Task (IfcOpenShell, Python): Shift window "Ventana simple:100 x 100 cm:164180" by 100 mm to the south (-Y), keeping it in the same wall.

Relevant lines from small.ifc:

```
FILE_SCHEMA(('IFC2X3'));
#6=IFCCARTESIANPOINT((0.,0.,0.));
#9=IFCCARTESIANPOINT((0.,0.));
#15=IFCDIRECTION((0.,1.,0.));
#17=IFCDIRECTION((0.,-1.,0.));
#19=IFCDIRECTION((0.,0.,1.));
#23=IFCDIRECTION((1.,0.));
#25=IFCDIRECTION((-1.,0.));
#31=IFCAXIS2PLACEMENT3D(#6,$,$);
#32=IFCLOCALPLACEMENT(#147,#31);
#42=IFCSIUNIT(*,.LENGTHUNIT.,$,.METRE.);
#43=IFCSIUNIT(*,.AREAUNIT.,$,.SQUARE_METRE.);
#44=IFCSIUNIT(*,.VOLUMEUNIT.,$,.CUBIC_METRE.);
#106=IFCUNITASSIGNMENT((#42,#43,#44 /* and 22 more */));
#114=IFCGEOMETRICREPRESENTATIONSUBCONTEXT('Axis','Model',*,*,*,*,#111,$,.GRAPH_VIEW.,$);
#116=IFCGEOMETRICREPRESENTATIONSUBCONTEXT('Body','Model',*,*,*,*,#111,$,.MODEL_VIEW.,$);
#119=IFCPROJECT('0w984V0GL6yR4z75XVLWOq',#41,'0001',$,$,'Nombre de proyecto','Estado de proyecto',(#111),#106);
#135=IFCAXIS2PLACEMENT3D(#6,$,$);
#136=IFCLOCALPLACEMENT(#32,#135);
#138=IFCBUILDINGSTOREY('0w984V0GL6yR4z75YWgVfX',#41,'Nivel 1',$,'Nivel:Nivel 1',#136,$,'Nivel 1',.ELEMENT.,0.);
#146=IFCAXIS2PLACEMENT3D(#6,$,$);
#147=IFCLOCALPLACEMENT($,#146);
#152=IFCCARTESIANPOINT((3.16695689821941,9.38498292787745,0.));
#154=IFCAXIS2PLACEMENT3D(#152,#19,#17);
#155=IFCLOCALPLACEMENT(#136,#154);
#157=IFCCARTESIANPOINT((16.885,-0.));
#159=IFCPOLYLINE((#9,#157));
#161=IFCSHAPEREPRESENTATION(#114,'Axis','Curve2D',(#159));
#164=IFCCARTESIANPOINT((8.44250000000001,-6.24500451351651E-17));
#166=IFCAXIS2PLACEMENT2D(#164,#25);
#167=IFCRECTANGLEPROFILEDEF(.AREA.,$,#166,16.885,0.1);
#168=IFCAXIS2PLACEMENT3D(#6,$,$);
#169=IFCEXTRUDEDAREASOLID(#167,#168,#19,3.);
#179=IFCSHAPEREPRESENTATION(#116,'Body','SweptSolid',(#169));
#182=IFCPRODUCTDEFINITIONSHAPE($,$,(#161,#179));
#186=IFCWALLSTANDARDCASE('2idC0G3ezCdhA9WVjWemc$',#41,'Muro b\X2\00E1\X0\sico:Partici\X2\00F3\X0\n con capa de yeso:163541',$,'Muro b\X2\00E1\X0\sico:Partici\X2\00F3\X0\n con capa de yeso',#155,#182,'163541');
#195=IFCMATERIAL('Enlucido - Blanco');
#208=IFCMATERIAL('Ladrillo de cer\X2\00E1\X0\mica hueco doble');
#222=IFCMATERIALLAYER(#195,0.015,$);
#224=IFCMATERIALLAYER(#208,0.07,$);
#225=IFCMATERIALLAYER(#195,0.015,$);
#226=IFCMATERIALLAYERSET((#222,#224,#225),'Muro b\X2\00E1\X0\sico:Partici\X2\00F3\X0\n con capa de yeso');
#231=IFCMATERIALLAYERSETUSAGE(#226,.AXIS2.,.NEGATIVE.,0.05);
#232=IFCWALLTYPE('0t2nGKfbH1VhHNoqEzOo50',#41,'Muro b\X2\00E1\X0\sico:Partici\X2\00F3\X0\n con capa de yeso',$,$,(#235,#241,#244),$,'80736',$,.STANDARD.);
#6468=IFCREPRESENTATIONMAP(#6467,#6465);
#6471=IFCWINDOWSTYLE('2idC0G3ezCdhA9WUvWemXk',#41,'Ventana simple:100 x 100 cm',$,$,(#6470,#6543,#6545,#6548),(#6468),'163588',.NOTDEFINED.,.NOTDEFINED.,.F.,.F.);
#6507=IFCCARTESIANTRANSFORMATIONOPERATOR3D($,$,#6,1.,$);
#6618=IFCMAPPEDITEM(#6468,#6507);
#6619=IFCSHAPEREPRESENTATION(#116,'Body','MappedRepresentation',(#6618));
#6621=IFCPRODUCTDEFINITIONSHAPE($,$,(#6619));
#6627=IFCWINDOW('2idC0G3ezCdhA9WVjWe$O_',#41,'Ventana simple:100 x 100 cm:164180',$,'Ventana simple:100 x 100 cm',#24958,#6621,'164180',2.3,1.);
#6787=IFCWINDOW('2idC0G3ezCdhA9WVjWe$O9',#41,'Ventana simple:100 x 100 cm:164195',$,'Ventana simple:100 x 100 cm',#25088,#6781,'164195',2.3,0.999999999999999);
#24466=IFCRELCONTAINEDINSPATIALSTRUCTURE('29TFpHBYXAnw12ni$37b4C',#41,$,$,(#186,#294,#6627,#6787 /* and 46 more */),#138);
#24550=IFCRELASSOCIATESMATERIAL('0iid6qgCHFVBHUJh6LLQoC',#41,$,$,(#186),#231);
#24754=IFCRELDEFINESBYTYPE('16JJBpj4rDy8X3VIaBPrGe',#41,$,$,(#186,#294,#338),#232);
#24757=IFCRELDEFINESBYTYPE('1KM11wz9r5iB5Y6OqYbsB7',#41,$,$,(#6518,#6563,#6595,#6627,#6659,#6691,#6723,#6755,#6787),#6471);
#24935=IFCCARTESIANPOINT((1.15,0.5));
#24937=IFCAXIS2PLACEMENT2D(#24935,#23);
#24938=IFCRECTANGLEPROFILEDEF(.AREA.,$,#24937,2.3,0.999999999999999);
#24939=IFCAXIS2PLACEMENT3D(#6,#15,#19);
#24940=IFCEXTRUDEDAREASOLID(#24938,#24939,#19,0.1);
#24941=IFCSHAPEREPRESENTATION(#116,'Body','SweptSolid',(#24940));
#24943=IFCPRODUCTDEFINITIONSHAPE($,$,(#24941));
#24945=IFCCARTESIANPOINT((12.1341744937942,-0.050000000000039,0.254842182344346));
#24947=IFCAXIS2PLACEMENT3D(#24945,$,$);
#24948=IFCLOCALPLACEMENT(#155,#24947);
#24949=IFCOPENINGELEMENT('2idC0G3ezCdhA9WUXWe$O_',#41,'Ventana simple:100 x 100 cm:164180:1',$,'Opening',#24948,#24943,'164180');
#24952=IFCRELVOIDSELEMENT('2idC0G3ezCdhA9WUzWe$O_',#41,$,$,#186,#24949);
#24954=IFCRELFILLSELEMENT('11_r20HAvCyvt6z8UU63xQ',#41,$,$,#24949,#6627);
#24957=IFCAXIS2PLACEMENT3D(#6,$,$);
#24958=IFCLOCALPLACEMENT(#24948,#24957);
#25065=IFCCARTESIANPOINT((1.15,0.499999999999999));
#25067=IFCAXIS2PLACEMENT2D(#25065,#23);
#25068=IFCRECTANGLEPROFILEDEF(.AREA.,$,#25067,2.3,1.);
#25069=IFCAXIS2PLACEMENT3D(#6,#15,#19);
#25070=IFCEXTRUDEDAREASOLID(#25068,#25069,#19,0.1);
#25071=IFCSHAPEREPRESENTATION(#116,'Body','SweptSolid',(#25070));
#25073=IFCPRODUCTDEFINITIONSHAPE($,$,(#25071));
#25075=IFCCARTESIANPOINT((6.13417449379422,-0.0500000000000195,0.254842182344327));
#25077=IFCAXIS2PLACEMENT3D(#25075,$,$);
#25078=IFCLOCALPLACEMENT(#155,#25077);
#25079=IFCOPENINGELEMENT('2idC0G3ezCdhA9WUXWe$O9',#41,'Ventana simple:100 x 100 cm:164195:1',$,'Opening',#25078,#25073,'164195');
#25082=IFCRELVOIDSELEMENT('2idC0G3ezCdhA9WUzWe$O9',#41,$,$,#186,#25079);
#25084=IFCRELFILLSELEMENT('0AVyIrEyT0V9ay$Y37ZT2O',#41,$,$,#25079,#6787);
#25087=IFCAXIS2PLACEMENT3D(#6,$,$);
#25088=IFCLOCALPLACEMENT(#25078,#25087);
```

```python
import ifcopenshell
import ifcopenshell.api.geometry
import ifcopenshell.util.placement

model = ifcopenshell.open("small.ifc")

window = model.by_guid("2idC0G3ezCdhA9WVjWe$O_")
opening = window.FillsVoids[0].RelatingOpeningElement
wall = opening.VoidsElements[0].RelatingBuildingElement

wall_matrix = ifcopenshell.util.placement.get_local_placement(wall.ObjectPlacement)
shift = wall_matrix[:3, 0] * 0.1
before = ifcopenshell.util.placement.get_local_placement(window.ObjectPlacement)[:3, 3].copy()

# The window is placed relative to its opening, so it follows when the opening moves.
matrix = ifcopenshell.util.placement.get_local_placement(opening.ObjectPlacement)
matrix[:3, 3] += shift
ifcopenshell.api.geometry.edit_object_placement(
    model, product=opening, matrix=matrix, is_si=False, should_transform_children=True
)

after = ifcopenshell.util.placement.get_local_placement(window.ObjectPlacement)[:3, 3]
print("window moved by", (after - before).round(3) + 0.0)

model.write("small_v2.ifc")
```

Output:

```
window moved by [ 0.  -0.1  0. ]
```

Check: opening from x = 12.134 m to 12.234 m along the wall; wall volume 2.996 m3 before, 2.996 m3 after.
